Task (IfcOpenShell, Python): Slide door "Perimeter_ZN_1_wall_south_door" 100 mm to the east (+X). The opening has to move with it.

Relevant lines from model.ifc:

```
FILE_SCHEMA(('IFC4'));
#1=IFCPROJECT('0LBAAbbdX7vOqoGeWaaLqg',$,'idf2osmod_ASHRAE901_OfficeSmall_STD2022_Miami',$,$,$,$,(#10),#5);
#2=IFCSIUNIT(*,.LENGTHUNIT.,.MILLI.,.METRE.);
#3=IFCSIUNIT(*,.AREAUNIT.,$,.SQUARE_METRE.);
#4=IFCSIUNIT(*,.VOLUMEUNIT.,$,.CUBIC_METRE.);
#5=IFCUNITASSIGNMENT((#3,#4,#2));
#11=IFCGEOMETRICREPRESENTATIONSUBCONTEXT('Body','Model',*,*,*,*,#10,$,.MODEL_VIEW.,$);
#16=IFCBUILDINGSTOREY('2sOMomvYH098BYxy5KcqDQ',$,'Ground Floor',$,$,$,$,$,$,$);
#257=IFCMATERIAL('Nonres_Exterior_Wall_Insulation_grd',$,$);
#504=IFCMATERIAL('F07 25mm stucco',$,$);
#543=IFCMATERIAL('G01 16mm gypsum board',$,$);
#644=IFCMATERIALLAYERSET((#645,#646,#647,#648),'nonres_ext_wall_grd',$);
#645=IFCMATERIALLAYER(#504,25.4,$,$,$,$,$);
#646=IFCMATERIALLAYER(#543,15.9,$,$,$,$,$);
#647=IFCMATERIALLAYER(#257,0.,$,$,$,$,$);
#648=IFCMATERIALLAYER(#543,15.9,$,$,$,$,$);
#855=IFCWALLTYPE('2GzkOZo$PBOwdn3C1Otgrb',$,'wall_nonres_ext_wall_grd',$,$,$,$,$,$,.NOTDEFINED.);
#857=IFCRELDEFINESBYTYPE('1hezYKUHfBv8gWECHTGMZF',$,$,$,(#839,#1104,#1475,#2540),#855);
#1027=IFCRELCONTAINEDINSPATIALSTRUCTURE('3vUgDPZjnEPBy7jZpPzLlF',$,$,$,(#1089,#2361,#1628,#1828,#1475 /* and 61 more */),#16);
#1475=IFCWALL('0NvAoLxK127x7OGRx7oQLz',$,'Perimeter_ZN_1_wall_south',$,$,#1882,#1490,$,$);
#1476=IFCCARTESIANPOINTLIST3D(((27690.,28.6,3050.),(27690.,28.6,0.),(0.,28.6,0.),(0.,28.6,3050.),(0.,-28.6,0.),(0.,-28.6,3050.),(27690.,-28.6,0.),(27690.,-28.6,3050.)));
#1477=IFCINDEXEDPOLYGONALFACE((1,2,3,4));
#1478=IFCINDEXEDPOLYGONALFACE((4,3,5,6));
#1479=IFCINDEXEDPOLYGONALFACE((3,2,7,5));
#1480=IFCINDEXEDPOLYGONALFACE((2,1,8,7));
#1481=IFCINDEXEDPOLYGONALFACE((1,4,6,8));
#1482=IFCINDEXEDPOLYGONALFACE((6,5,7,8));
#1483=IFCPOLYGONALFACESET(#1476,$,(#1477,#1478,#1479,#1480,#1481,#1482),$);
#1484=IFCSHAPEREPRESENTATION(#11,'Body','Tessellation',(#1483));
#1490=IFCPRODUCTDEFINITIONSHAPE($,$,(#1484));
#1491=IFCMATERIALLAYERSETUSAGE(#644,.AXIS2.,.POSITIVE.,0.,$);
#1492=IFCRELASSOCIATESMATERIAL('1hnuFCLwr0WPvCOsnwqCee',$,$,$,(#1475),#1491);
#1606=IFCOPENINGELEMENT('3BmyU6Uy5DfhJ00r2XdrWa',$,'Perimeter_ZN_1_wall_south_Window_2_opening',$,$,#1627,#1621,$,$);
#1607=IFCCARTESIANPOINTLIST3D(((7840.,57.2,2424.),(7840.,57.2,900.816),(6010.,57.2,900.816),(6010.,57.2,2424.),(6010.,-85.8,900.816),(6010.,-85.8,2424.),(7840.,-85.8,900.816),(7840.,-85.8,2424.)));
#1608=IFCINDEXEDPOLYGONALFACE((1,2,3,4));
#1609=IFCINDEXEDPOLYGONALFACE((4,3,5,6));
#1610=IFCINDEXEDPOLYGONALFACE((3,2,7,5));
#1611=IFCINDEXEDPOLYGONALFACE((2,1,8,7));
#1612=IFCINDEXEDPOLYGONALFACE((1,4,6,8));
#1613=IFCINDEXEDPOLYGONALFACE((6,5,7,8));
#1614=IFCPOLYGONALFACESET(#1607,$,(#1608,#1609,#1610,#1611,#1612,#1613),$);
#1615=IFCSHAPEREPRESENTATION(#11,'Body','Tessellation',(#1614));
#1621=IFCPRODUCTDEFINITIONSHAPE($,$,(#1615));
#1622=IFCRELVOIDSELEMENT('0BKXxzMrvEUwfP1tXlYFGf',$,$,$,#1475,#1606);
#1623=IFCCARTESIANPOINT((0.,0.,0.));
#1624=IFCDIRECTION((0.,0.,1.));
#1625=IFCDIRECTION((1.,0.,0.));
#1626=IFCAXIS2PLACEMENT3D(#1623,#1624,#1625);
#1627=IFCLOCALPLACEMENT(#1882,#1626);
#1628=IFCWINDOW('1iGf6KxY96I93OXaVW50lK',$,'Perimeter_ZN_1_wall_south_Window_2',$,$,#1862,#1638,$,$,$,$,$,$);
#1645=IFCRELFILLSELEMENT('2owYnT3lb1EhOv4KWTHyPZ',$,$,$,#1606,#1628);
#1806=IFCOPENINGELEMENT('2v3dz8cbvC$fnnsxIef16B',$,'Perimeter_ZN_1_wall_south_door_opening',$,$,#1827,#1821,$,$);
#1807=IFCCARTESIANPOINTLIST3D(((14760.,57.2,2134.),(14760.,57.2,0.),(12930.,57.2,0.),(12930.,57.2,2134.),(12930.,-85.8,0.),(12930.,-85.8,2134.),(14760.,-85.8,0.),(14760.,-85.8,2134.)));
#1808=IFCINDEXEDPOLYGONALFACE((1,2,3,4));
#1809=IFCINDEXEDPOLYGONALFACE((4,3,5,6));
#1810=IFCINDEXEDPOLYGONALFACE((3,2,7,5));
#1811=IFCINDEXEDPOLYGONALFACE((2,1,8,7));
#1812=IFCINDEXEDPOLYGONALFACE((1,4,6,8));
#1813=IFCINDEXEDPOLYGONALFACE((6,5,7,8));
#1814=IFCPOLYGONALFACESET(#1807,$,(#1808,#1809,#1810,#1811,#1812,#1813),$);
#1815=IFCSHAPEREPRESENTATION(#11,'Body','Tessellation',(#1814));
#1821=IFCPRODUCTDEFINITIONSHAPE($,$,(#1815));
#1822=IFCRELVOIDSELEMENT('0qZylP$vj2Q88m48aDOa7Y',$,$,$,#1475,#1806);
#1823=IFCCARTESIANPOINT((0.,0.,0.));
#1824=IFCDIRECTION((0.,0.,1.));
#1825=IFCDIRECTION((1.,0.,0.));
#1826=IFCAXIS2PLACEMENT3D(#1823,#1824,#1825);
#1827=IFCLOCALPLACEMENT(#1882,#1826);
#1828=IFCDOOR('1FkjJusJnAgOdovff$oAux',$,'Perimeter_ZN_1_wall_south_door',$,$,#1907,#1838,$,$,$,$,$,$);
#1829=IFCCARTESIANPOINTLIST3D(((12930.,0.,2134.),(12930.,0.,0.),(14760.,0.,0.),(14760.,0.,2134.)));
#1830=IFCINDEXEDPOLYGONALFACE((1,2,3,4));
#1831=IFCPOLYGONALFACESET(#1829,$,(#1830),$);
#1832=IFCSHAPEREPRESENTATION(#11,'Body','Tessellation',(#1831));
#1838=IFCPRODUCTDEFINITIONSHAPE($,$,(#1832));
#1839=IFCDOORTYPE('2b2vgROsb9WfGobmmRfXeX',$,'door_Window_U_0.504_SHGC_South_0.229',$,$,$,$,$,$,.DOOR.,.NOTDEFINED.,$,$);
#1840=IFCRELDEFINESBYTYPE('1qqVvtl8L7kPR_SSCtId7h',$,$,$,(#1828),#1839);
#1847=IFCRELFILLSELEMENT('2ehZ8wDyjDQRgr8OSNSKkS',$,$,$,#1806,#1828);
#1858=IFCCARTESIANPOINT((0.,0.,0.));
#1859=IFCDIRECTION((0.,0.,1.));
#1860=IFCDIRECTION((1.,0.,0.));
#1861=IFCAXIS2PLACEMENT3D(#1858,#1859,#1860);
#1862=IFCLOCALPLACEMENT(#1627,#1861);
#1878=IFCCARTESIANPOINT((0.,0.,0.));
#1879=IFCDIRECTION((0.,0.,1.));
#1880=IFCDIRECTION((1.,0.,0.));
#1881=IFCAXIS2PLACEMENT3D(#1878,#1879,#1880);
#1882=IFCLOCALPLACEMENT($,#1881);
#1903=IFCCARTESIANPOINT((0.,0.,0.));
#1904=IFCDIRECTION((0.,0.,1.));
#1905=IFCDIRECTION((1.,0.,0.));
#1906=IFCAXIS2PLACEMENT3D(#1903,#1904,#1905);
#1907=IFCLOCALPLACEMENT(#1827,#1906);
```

```python
import ifcopenshell
import ifcopenshell.api.geometry
import ifcopenshell.util.placement
import ifcopenshell.util.unit

model = ifcopenshell.open("model.ifc")
unit_scale = ifcopenshell.util.unit.calculate_unit_scale(model)

door = model.by_guid("1FkjJusJnAgOdovff$oAux")
opening = door.FillsVoids[0].RelatingOpeningElement
wall = opening.VoidsElements[0].RelatingBuildingElement

wall_matrix = ifcopenshell.util.placement.get_local_placement(wall.ObjectPlacement)
shift = wall_matrix[:3, 0] * 0.1 / unit_scale
before = ifcopenshell.util.placement.get_local_placement(door.ObjectPlacement)[:3, 3].copy()

# The door is placed relative to its opening, so it follows when the opening moves.
matrix = ifcopenshell.util.placement.get_local_placement(opening.ObjectPlacement)
matrix[:3, 3] += shift
ifcopenshell.api.geometry.edit_object_placement(
    model, product=opening, matrix=matrix, is_si=False, should_transform_children=True
)

after = ifcopenshell.util.placement.get_local_placement(door.ObjectPlacement)[:3, 3]
print("door moved by", (after - before).round(3) + 0.0)

model.write("model_v2.ifc")
```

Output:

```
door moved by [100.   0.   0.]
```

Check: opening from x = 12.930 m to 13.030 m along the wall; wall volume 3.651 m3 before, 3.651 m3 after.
